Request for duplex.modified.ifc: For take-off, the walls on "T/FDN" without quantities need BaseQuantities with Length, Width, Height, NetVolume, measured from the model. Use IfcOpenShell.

First a look at what the model holds.

```python
import ifcopenshell
import ifcopenshell.util.element
import ifcopenshell.util.unit

model = ifcopenshell.open("duplex.modified.ifc")
print(model.schema)
for unit_type in ("LENGTHUNIT", "AREAUNIT", "VOLUMEUNIT"):
    print(unit_type, ifcopenshell.util.unit.calculate_unit_scale(model, unit_type))
storey = next(s for s in model.by_type("IfcBuildingStorey") if s.Name == "T/FDN")
walls = [e for e in ifcopenshell.util.element.get_decomposition(storey) if e.is_a("IfcWall")]
for e in sorted(walls, key=lambda e: e.id()):
    print(e.id(), e.is_a(), e.Name, list(ifcopenshell.util.element.get_psets(e, qtos_only=True)), sep=" | ")
```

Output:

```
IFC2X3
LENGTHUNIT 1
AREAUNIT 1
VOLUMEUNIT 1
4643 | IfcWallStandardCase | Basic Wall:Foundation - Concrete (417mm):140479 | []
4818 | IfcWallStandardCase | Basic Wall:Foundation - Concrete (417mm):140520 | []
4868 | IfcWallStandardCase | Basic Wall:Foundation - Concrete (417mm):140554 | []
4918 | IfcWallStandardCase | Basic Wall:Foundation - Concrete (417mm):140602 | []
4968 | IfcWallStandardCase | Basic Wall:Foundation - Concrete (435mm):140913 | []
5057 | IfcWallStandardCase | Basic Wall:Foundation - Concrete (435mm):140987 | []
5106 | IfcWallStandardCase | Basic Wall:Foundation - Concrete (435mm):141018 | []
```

```python
import ifcopenshell
import ifcopenshell.api.pset
import ifcopenshell.geom
import ifcopenshell.util.element
import ifcopenshell.util.shape
import ifcopenshell.util.unit

model = ifcopenshell.open("duplex.modified.ifc")
unit_scale = ifcopenshell.util.unit.calculate_unit_scale(model)
volume_scale = ifcopenshell.util.unit.calculate_unit_scale(model, "VOLUMEUNIT")
settings = ifcopenshell.geom.settings()

storey = next(s for s in model.by_type("IfcBuildingStorey") if s.Name == "T/FDN")
walls = [e for e in ifcopenshell.util.element.get_decomposition(storey) if e.is_a("IfcWall")]

for e in sorted(walls, key=lambda e: e.id()):
    if ifcopenshell.util.element.get_psets(e, qtos_only=True, should_inherit=False):
        continue
    # Geometry comes back in metres, in the element's own axes.
    shape = ifcopenshell.geom.create_shape(settings, e)
    values = {
        "Length": ifcopenshell.util.shape.get_x(shape.geometry) / unit_scale,
        "Width": ifcopenshell.util.shape.get_y(shape.geometry) / unit_scale,
        "Height": ifcopenshell.util.shape.get_z(shape.geometry) / unit_scale,
        "NetVolume": ifcopenshell.util.shape.get_volume(shape.geometry) / volume_scale,
    }
    qto = ifcopenshell.api.pset.add_qto(model, product=e, name="BaseQuantities")
    ifcopenshell.api.pset.edit_qto(model, qto=qto, properties=values)
    print(e.id(), {k: round(v, 3) for k, v in values.items()})

model.write("duplex.modified-out.ifc")
```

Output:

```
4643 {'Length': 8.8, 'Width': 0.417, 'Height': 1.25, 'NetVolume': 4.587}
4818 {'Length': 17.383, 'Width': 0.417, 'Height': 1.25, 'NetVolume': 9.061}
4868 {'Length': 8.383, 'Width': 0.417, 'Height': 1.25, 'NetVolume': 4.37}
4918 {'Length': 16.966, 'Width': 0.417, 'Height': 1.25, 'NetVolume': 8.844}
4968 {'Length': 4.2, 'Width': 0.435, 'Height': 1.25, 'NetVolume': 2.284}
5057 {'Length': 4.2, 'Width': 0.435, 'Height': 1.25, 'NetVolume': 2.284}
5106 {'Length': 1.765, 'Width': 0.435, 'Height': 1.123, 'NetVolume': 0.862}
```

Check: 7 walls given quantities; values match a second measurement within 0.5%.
